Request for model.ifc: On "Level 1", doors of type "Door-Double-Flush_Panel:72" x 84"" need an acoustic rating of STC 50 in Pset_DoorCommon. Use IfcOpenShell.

First a look at what the model holds.

```python
import ifcopenshell
import ifcopenshell.util.element

model = ifcopenshell.open("model.ifc")
print(model.schema)
storey = next(s for s in model.by_type("IfcBuildingStorey") if s.Name == "Level 1")
doors = [e for e in ifcopenshell.util.element.get_decomposition(storey) if e.is_a("IfcDoor")]
seen = {}
for e in doors:
    element_type = ifcopenshell.util.element.get_type(e)
    key = (element_type.Name if element_type != e and element_type else None, ifcopenshell.util.element.get_pset(e, "Pset_DoorCommon", "AcousticRating"))
    seen[key] = seen.get(key, 0) + 1
for (name, value), count in sorted(seen.items(), key=str):
    print(count, "x", name, "|", value)
```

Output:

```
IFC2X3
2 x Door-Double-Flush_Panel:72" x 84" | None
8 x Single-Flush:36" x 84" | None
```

```python
import ifcopenshell
import ifcopenshell.api.pset
import ifcopenshell.util.element

model = ifcopenshell.open("model.ifc")

storey = next(s for s in model.by_type("IfcBuildingStorey") if s.Name == "Level 1")
doors = [e for e in ifcopenshell.util.element.get_decomposition(storey) if e.is_a("IfcDoor")]

count = 0
for e in doors:
    element_type = ifcopenshell.util.element.get_type(e)
    if element_type in (None, e) or element_type.Name != 'Door-Double-Flush_Panel:72" x 84"':
        continue
    # add_pset returns the element's existing set when there is one.
    pset = ifcopenshell.api.pset.add_pset(model, product=e, name="Pset_DoorCommon")
    ifcopenshell.api.pset.edit_pset(model, pset=pset, properties={"AcousticRating": "STC 50"})
    count += 1

print(count, "doors updated")

model.write("model_updated.ifc")
```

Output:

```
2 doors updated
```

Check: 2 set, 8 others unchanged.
